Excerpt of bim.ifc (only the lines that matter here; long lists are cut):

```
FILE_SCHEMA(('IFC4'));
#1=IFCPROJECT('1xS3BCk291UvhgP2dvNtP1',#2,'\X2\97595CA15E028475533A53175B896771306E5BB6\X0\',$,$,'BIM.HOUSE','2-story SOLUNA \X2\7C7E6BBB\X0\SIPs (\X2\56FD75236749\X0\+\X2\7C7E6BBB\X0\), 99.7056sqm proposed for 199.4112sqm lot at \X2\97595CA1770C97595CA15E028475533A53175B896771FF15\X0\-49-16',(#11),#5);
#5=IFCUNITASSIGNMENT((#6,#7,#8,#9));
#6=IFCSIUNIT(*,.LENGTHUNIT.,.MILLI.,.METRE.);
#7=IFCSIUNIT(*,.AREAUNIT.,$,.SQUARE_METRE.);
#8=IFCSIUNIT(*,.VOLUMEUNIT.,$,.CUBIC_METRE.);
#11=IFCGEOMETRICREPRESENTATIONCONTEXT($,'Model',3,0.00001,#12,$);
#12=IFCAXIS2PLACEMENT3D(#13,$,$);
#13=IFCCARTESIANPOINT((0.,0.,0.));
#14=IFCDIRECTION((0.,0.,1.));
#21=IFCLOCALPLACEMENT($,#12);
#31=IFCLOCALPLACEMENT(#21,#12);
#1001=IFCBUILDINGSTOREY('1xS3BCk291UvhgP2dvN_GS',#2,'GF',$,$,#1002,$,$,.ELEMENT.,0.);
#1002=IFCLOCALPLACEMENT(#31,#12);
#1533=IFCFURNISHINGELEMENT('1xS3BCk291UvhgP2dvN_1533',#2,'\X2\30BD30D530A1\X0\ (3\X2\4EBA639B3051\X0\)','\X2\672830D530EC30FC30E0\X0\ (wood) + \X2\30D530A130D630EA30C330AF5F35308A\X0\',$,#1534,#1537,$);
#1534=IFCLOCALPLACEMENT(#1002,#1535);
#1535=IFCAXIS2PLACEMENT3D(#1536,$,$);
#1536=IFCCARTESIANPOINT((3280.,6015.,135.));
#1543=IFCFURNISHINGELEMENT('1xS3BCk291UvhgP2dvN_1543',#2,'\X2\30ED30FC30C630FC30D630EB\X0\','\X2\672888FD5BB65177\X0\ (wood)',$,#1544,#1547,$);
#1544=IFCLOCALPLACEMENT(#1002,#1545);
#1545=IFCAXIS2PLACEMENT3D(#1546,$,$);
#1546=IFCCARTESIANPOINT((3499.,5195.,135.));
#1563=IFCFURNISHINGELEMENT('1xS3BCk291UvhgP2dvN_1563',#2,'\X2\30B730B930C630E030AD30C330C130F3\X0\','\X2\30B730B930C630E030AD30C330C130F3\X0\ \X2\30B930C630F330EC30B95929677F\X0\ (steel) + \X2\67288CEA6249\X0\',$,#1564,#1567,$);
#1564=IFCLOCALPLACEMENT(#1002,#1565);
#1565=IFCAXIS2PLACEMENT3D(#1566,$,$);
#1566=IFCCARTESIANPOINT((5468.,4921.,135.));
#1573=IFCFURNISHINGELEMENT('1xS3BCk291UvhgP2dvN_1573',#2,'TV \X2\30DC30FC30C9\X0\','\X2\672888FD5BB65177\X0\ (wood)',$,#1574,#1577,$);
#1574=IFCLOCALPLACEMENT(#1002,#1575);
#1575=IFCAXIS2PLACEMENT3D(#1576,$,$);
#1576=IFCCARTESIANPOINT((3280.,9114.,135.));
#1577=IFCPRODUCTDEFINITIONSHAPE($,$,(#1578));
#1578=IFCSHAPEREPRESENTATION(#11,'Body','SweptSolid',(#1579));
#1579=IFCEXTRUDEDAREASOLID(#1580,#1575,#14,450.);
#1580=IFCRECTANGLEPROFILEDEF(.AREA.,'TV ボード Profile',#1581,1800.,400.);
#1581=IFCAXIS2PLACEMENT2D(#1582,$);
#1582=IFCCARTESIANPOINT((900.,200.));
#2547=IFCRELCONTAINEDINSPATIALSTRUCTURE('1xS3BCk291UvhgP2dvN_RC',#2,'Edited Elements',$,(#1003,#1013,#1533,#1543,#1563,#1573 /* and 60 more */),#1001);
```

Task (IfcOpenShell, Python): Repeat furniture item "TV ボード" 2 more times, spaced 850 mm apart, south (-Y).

```python
import numpy as np
import ifcopenshell
import ifcopenshell.api.geometry
import ifcopenshell.api.root
import ifcopenshell.util.element
import ifcopenshell.util.placement
import ifcopenshell.util.unit

model = ifcopenshell.open("bim.ifc")
unit_scale = ifcopenshell.util.unit.calculate_unit_scale(model)


def reuse_history(source, copy):
    """copy_class also copies each property set's owner history, people and application; keep the originals."""
    for rel in copy.IsDefinedBy:
        if rel.is_a("IfcRelDefinesByProperties") and (history := rel.RelatingPropertyDefinition.OwnerHistory):
            rel.RelatingPropertyDefinition.OwnerHistory = source.OwnerHistory
            ifcopenshell.util.element.remove_deep2(model, history)


source = model.by_guid("1xS3BCk291UvhgP2dvN_1573")
base = ifcopenshell.util.placement.get_local_placement(source.ObjectPlacement)
step = np.array([0.0, -1.0, 0.0]) * 0.85 / unit_scale

for i in range(1, 3):
    copy = ifcopenshell.api.root.copy_class(model, product=source)
    copy.Representation = ifcopenshell.util.element.copy_deep(
        model, source.Representation, exclude=["IfcGeometricRepresentationContext", "IfcRepresentationMap"]
    )
    reuse_history(source, copy)
    matrix = base.copy()
    matrix[:3, 3] += i * step
    print("added at", matrix[:3, 3].round(3) + 0.0)
    ifcopenshell.api.geometry.edit_object_placement(model, product=copy, matrix=matrix, is_si=False)

model.write("bim_rev.ifc")
```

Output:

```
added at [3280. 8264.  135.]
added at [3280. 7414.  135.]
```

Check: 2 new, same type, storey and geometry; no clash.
